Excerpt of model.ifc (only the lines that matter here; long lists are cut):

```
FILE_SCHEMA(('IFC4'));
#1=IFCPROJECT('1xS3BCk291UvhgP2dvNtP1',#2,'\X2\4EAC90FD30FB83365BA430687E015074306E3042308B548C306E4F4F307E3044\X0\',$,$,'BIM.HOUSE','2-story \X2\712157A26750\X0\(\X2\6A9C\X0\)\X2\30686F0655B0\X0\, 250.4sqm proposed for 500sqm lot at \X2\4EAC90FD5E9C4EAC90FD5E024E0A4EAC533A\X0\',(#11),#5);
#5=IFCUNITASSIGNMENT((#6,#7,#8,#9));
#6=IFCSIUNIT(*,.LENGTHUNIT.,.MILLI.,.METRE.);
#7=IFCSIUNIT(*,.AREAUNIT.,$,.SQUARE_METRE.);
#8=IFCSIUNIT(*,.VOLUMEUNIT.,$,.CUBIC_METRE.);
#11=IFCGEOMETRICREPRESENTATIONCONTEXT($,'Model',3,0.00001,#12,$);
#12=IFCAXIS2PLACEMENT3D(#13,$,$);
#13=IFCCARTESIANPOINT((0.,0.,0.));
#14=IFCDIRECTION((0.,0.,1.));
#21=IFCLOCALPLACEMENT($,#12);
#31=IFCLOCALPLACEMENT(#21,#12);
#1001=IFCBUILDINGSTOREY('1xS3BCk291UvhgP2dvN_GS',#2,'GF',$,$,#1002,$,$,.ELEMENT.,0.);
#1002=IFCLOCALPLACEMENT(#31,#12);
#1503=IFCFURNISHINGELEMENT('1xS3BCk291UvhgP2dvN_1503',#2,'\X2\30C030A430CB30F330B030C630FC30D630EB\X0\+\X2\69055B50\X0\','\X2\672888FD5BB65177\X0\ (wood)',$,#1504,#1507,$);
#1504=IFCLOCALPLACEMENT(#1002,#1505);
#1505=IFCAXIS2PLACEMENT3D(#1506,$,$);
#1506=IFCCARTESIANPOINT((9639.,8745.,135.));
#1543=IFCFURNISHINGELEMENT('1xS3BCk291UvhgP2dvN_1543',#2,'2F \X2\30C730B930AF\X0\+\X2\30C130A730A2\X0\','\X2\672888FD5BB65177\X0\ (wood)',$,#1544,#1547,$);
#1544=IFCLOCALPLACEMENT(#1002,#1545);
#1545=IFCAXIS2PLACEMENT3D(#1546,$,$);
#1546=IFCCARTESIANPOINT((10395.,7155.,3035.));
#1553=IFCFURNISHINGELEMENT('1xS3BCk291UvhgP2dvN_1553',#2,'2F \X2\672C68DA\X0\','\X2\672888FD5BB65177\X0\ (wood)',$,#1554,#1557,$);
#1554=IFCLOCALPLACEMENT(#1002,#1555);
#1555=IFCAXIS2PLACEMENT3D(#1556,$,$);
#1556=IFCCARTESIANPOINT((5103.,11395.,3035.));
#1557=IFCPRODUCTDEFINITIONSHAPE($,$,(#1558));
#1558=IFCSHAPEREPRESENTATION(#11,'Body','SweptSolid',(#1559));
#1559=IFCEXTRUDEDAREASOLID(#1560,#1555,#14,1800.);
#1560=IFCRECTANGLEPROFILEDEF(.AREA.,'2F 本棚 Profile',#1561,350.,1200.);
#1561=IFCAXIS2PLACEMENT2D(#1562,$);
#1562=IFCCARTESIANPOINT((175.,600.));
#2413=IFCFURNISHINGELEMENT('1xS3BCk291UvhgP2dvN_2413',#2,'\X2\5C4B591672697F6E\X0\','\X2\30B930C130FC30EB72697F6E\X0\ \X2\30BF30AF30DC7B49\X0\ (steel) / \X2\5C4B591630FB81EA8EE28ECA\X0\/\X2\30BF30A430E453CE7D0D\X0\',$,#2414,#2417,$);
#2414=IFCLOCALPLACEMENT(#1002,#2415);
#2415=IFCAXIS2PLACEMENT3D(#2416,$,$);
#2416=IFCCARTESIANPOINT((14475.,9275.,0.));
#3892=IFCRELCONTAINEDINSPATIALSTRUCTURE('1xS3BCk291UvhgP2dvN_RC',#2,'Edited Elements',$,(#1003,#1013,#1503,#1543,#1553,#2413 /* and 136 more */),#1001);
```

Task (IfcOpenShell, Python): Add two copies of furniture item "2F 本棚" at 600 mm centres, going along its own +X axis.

```python
import ifcopenshell
import ifcopenshell.api.geometry
import ifcopenshell.api.root
import ifcopenshell.util.element
import ifcopenshell.util.placement
import ifcopenshell.util.unit

model = ifcopenshell.open("model.ifc")
unit_scale = ifcopenshell.util.unit.calculate_unit_scale(model)


def reuse_history(source, copy):
    """copy_class also copies each property set's owner history, people and application; keep the originals."""
    for rel in copy.IsDefinedBy:
        if rel.is_a("IfcRelDefinesByProperties") and (history := rel.RelatingPropertyDefinition.OwnerHistory):
            rel.RelatingPropertyDefinition.OwnerHistory = source.OwnerHistory
            ifcopenshell.util.element.remove_deep2(model, history)


source = model.by_guid("1xS3BCk291UvhgP2dvN_1553")
base = ifcopenshell.util.placement.get_local_placement(source.ObjectPlacement)
step = base[:3, 0] * 0.6 / unit_scale

for i in range(1, 3):
    copy = ifcopenshell.api.root.copy_class(model, product=source)
    copy.Representation = ifcopenshell.util.element.copy_deep(
        model, source.Representation, exclude=["IfcGeometricRepresentationContext", "IfcRepresentationMap"]
    )
    reuse_history(source, copy)
    matrix = base.copy()
    matrix[:3, 3] += i * step
    print("added at", matrix[:3, 3].round(3) + 0.0)
    ifcopenshell.api.geometry.edit_object_placement(model, product=copy, matrix=matrix, is_si=False)

model.write("model_v2.ifc")
```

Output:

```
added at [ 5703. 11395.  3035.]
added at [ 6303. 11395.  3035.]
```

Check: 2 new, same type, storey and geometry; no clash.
